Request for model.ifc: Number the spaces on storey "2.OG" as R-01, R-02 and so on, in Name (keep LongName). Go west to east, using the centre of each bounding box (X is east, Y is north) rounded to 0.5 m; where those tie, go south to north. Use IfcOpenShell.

First a look at what the model holds.

```python
import ifcopenshell
import ifcopenshell.util.element
import ifcopenshell.util.placement

model = ifcopenshell.open("model.ifc")
print(model.schema)
storey = next(s for s in model.by_type("IfcBuildingStorey") if s.Name == "2.OG")
spaces = [e for e in ifcopenshell.util.element.get_decomposition(storey) if e.is_a("IfcSpace")]
for e in sorted(spaces, key=lambda e: e.id()):
    origin = ifcopenshell.util.placement.get_local_placement(e.ObjectPlacement)[:3, 3]
    print(e.id(), e.Name, e.LongName, origin.round(2) + 0.0, sep=" | ")
```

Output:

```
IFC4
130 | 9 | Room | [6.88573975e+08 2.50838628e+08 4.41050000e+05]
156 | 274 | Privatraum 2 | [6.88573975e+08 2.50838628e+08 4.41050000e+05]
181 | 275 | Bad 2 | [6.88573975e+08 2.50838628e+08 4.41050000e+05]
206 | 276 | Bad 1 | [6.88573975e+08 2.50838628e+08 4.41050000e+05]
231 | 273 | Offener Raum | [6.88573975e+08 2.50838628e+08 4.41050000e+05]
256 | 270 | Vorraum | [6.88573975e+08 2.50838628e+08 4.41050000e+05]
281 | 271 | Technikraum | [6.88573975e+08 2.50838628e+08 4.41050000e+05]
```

```python
import ifcopenshell
import ifcopenshell.geom
import ifcopenshell.util.element
import ifcopenshell.util.shape

model = ifcopenshell.open("model.ifc")
settings = ifcopenshell.geom.settings()
settings.set("use-world-coords", True)


def centre(element):
    shape = ifcopenshell.geom.create_shape(settings, element)
    return ifcopenshell.util.shape.get_bbox_centroid(shape.geometry)


storey = next(s for s in model.by_type("IfcBuildingStorey") if s.Name == "2.OG")
spaces = [e for e in ifcopenshell.util.element.get_decomposition(storey) if e.is_a("IfcSpace")]

# Insertion points can sit at a corner or the storey origin, so sort by the geometry (in metres).
centres = {e: centre(e) for e in spaces}
spaces.sort(key=lambda e: (round(centres[e][0] / 0.5), centres[e][1]))

for i, e in enumerate(spaces, start=1):
    number = f"R-{i:02d}"
    e.Name = number
    print(e.id(), number)

model.write("model-out.ifc")
```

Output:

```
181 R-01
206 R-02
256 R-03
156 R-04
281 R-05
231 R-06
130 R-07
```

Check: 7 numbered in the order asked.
